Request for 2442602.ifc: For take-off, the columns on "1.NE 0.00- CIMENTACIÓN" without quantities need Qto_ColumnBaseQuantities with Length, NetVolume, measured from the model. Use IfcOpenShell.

First a look at what the model holds.

```python
import ifcopenshell
import ifcopenshell.util.element
import ifcopenshell.util.unit

model = ifcopenshell.open("2442602.ifc")
print(model.schema)
for unit_type in ("LENGTHUNIT", "AREAUNIT", "VOLUMEUNIT"):
    print(unit_type, ifcopenshell.util.unit.calculate_unit_scale(model, unit_type))
storey = next(s for s in model.by_type("IfcBuildingStorey") if s.Name == "1.NE 0.00- CIMENTACIÓN")
columns = [e for e in ifcopenshell.util.element.get_decomposition(storey) if e.is_a("IfcColumn")]
for e in sorted(columns, key=lambda e: e.id()):
    print(e.id(), e.is_a(), e.Name, list(ifcopenshell.util.element.get_psets(e, qtos_only=True)), sep=" | ")
```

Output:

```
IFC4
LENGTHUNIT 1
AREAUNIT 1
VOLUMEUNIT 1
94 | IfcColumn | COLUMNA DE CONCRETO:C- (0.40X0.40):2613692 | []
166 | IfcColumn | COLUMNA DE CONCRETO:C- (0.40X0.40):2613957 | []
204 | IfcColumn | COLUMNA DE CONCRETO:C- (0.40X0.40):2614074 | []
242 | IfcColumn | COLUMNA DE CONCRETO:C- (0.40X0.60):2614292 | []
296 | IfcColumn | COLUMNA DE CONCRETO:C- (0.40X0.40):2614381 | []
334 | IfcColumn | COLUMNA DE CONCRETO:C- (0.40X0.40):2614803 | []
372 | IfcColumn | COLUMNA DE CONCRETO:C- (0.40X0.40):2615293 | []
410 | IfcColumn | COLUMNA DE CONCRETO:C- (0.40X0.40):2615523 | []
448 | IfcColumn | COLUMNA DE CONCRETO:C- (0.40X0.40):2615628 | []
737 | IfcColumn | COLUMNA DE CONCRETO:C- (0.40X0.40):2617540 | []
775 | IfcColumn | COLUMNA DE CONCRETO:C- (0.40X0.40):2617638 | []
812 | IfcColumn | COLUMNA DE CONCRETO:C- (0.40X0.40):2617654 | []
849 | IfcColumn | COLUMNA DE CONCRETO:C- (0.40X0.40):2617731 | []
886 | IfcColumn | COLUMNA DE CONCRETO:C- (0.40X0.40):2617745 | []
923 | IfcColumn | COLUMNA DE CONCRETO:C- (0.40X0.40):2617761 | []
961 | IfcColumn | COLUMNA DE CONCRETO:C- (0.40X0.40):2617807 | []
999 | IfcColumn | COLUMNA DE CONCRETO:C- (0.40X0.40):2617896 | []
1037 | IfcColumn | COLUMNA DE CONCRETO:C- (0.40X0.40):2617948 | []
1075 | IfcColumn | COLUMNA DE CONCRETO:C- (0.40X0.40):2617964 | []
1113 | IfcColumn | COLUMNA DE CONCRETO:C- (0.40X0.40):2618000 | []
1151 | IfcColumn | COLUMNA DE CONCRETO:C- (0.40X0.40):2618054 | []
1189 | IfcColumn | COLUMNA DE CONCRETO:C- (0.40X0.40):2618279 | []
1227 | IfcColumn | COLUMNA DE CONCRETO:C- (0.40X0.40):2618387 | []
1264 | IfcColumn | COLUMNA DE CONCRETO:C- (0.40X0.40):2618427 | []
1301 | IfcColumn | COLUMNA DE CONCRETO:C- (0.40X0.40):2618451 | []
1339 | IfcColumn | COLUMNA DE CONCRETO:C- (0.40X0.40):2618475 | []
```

```python
import ifcopenshell
import ifcopenshell.api.pset
import ifcopenshell.geom
import ifcopenshell.util.element
import ifcopenshell.util.shape
import ifcopenshell.util.unit

model = ifcopenshell.open("2442602.ifc")
unit_scale = ifcopenshell.util.unit.calculate_unit_scale(model)
volume_scale = ifcopenshell.util.unit.calculate_unit_scale(model, "VOLUMEUNIT")
settings = ifcopenshell.geom.settings()

storey = next(s for s in model.by_type("IfcBuildingStorey") if s.Name == "1.NE 0.00- CIMENTACIÓN")
columns = [e for e in ifcopenshell.util.element.get_decomposition(storey) if e.is_a("IfcColumn")]

for e in sorted(columns, key=lambda e: e.id()):
    if ifcopenshell.util.element.get_psets(e, qtos_only=True, should_inherit=False):
        continue
    # Geometry comes back in metres, in the element's own axes.
    shape = ifcopenshell.geom.create_shape(settings, e)
    values = {
        "Length": ifcopenshell.util.shape.get_z(shape.geometry) / unit_scale,
        "NetVolume": ifcopenshell.util.shape.get_volume(shape.geometry) / volume_scale,
    }
    qto = ifcopenshell.api.pset.add_qto(model, product=e, name="Qto_ColumnBaseQuantities")
    ifcopenshell.api.pset.edit_qto(model, qto=qto, properties=values)
    print(e.id(), {k: round(v, 3) for k, v in values.items()})

model.write("2442602_rev.ifc")
```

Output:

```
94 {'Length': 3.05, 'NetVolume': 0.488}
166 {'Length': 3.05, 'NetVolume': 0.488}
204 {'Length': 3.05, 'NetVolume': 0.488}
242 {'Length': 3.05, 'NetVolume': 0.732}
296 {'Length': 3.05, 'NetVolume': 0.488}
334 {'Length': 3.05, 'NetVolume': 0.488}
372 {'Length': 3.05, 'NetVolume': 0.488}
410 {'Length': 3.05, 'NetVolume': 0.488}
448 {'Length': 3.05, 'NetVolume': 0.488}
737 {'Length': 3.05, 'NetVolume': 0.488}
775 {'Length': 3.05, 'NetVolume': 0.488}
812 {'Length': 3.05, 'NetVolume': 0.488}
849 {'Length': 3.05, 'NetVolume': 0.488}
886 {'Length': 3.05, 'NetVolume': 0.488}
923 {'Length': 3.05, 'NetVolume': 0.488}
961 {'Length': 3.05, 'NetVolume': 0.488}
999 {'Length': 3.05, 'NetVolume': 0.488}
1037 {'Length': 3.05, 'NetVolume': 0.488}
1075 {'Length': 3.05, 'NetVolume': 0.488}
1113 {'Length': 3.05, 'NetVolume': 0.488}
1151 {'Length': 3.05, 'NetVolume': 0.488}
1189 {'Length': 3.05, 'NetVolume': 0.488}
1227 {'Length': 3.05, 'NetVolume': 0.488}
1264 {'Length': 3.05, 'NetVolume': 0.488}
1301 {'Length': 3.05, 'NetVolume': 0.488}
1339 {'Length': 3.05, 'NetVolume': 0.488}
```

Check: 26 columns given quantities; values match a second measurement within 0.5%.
